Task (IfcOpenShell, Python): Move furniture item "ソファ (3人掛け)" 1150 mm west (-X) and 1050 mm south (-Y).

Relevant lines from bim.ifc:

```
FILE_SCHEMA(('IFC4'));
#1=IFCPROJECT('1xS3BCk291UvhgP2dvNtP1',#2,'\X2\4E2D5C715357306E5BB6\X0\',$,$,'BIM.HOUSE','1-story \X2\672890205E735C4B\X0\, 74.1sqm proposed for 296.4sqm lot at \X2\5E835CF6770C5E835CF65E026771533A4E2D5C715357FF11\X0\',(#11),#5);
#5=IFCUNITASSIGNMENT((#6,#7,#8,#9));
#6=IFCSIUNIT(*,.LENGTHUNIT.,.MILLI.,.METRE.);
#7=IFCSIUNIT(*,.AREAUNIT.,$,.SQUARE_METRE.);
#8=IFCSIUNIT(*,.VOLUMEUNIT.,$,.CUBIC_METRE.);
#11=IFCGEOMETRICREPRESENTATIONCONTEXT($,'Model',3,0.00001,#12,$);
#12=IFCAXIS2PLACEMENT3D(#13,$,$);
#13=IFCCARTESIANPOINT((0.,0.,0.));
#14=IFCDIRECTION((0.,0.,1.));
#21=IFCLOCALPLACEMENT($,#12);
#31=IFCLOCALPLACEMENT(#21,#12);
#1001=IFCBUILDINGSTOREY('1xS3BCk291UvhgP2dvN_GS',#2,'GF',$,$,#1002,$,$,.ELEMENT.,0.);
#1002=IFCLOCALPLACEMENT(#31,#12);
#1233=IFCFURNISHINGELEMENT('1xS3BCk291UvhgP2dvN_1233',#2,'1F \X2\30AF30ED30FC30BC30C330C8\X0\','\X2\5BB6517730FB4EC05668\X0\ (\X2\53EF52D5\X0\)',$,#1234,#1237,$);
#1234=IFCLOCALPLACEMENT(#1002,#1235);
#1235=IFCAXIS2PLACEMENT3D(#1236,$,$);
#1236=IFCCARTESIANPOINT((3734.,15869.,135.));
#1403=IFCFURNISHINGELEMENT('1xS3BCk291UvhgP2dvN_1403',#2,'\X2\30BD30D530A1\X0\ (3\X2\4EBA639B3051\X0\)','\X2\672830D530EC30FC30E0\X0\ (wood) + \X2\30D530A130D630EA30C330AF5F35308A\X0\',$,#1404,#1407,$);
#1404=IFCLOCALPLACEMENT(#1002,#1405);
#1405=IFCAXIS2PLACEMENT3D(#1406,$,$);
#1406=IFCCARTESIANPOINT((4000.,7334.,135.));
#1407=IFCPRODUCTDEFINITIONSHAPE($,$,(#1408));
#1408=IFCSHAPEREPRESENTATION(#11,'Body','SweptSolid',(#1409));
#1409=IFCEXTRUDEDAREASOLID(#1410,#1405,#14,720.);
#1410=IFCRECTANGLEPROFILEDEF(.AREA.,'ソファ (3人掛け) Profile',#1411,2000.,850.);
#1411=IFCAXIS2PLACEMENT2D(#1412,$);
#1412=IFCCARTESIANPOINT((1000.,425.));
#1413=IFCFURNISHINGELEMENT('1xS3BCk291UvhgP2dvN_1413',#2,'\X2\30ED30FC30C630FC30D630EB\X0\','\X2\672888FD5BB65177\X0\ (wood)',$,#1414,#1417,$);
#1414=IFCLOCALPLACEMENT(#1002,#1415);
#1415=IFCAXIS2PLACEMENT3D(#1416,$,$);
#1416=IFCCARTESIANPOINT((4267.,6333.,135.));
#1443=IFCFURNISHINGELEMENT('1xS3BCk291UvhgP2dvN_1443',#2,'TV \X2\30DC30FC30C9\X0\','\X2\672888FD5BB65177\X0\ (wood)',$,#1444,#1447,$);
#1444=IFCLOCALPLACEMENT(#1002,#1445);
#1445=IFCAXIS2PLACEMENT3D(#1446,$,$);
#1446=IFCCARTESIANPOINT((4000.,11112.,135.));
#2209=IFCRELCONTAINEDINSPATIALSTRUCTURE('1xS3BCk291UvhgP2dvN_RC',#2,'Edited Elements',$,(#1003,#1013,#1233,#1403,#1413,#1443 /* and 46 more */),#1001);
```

```python
import ifcopenshell
import ifcopenshell.api.geometry
import ifcopenshell.util.placement

model = ifcopenshell.open("bim.ifc")

item = model.by_id(1403)
matrix = ifcopenshell.util.placement.get_local_placement(item.ObjectPlacement)
matrix[0, 3] -= 1150.0
matrix[1, 3] -= 1050.0
ifcopenshell.api.geometry.edit_object_placement(model, product=item, matrix=matrix, is_si=False)

print(ifcopenshell.util.placement.get_local_placement(item.ObjectPlacement).round(3) + 0.0)

model.write("bim_updated.ifc")
```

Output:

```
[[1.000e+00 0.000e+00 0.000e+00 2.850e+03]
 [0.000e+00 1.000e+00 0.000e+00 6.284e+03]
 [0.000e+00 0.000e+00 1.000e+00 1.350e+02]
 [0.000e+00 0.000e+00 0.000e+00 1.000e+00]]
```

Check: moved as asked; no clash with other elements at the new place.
